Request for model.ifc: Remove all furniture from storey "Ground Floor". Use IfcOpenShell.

First a look at what the model holds.

```python
import ifcopenshell
import ifcopenshell.util.element

model = ifcopenshell.open("model.ifc")
print(model.schema)
storey = next(s for s in model.by_type("IfcBuildingStorey") if s.Name == "Ground Floor")
furniture = [e for e in ifcopenshell.util.element.get_decomposition(storey) if e.is_a("IfcFurnishingElement")]
seen = {}
for e in furniture:
    element_type = ifcopenshell.util.element.get_type(e)
    name = element_type.Name if element_type not in (None, e) else None
    seen[name] = seen.get(name, 0) + 1
for name, count in sorted(seen.items(), key=str):
    print(count, "x", name)
```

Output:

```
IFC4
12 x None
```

```python
import ifcopenshell
import ifcopenshell.api.root
import ifcopenshell.util.element

model = ifcopenshell.open("model.ifc")

storey = next(s for s in model.by_type("IfcBuildingStorey") if s.Name == "Ground Floor")
furniture = [e for e in ifcopenshell.util.element.get_decomposition(storey) if e.is_a("IfcFurnishingElement")]

for e in furniture:
    ifcopenshell.api.root.remove_product(model, product=e)
print(len(furniture), "removed")

model.write("model_v2.ifc")
```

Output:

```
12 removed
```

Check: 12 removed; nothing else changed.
